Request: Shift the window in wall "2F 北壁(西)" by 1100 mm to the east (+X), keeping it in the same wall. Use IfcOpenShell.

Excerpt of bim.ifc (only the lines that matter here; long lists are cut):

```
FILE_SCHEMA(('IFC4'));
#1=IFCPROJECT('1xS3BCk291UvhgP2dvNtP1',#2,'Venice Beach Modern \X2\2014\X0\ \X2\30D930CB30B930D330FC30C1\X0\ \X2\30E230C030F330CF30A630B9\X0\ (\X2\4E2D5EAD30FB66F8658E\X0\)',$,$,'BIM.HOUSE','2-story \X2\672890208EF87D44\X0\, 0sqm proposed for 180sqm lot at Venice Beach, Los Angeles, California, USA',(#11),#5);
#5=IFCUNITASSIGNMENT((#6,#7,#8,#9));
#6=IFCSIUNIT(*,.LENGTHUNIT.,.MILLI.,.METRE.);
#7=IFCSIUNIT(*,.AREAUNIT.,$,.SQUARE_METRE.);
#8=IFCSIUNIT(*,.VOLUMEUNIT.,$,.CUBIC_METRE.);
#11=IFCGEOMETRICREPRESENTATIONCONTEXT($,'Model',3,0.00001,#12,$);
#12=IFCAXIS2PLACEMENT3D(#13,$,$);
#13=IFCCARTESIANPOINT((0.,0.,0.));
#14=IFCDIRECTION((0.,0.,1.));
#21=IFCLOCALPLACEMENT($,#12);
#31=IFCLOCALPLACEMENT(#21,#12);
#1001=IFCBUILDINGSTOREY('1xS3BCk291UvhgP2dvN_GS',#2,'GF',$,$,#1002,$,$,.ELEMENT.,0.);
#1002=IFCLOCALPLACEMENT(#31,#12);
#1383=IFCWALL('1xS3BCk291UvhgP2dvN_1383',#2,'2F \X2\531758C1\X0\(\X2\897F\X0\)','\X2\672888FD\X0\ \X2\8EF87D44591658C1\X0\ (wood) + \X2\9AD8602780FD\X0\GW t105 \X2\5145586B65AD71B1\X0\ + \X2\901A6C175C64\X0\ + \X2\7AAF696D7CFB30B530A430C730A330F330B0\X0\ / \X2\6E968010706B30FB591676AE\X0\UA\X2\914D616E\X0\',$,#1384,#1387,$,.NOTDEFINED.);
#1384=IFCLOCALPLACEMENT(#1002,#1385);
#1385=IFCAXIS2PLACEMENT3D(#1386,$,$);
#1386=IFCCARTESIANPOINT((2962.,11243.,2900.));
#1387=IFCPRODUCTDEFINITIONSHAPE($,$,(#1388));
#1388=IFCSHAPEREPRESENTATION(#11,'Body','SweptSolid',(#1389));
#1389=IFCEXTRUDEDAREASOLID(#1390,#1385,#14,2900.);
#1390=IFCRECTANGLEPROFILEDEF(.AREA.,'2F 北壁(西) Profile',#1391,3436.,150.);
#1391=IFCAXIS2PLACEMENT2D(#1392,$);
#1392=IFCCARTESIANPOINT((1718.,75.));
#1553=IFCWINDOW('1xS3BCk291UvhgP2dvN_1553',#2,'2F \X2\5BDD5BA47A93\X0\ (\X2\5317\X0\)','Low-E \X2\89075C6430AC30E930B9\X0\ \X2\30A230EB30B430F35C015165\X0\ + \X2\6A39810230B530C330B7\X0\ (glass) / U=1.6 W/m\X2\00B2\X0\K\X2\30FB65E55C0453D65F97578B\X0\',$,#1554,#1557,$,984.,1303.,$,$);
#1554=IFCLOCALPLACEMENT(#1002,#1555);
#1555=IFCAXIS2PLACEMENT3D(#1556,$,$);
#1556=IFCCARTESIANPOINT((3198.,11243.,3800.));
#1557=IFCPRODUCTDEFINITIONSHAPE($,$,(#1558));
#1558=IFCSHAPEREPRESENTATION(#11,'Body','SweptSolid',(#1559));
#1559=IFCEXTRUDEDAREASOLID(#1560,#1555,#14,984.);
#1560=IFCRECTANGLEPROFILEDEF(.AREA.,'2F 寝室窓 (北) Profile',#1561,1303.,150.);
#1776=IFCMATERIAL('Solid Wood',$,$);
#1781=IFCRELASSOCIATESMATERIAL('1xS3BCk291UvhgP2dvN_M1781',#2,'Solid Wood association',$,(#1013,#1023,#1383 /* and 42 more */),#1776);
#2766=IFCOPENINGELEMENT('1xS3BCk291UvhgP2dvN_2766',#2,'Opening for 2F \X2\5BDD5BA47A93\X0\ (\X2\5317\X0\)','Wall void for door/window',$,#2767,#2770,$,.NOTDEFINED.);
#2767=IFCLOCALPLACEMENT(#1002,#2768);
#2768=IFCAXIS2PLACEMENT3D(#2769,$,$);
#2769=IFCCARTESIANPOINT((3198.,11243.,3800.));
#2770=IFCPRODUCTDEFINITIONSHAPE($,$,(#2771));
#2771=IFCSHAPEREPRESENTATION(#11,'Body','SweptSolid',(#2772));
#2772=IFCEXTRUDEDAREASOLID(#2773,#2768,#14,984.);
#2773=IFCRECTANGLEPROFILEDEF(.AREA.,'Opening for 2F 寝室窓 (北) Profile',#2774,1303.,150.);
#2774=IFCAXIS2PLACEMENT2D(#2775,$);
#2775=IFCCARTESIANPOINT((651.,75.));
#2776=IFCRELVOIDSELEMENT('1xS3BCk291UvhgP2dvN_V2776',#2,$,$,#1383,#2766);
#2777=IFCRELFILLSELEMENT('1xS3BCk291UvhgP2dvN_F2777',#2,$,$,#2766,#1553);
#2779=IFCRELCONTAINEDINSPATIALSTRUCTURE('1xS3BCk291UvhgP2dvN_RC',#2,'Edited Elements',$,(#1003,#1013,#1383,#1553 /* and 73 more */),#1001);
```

```python
import ifcopenshell
import ifcopenshell.api.geometry
import ifcopenshell.util.placement

model = ifcopenshell.open("bim.ifc")

window = model.by_guid("1xS3BCk291UvhgP2dvN_1553")
opening = window.FillsVoids[0].RelatingOpeningElement
wall = opening.VoidsElements[0].RelatingBuildingElement

wall_matrix = ifcopenshell.util.placement.get_local_placement(wall.ObjectPlacement)
shift = wall_matrix[:3, 0] * 1100.0
before = ifcopenshell.util.placement.get_local_placement(window.ObjectPlacement)[:3, 3].copy()

# The window is not placed relative to its opening, so move both.
for product in (opening, window):
    matrix = ifcopenshell.util.placement.get_local_placement(product.ObjectPlacement)
    matrix[:3, 3] += shift
    ifcopenshell.api.geometry.edit_object_placement(model, product=product, matrix=matrix, is_si=False)

after = ifcopenshell.util.placement.get_local_placement(window.ObjectPlacement)[:3, 3]
print("window moved by", (after - before).round(3) + 0.0)

model.write("bim_rev.ifc")
```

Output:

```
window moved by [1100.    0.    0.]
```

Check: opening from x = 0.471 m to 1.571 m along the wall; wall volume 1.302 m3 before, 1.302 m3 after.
